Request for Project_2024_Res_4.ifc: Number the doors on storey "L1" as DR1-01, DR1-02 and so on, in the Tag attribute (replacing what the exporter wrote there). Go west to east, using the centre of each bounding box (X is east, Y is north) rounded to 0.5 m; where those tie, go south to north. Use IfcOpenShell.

First a look at what the model holds.

```python
import ifcopenshell
import ifcopenshell.util.element
import ifcopenshell.util.placement

model = ifcopenshell.open("Project_2024_Res_4.ifc")
print(model.schema)
storey = next(s for s in model.by_type("IfcBuildingStorey") if s.Name == "L1")
doors = [e for e in ifcopenshell.util.element.get_decomposition(storey) if e.is_a("IfcDoor")]
for e in sorted(doors, key=lambda e: e.id()):
    origin = ifcopenshell.util.placement.get_local_placement(e.ObjectPlacement)[:3, 3]
    print(e.id(), e.Tag, e.Name, origin.round(2) + 0.0, sep=" | ")
```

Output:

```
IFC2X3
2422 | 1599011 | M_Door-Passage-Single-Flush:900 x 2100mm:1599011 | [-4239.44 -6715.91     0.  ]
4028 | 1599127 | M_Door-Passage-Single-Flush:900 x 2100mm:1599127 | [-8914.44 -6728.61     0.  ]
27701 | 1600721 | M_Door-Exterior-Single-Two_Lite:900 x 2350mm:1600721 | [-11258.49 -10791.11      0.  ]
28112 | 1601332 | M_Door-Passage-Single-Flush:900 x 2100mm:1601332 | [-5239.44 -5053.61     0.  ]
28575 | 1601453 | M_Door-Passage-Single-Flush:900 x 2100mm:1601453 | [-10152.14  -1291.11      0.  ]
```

```python
import ifcopenshell
import ifcopenshell.geom
import ifcopenshell.util.element
import ifcopenshell.util.shape

model = ifcopenshell.open("Project_2024_Res_4.ifc")
settings = ifcopenshell.geom.settings()
settings.set("use-world-coords", True)


def centre(element):
    shape = ifcopenshell.geom.create_shape(settings, element)
    return ifcopenshell.util.shape.get_bbox_centroid(shape.geometry)


storey = next(s for s in model.by_type("IfcBuildingStorey") if s.Name == "L1")
doors = [e for e in ifcopenshell.util.element.get_decomposition(storey) if e.is_a("IfcDoor")]

# Insertion points can sit at a corner or the storey origin, so sort by the geometry (in metres).
centres = {e: centre(e) for e in doors}
doors.sort(key=lambda e: (round(centres[e][0] / 0.5), centres[e][1]))

for i, e in enumerate(doors, start=1):
    number = f"DR1-{i:02d}"
    e.Tag = number
    print(e.id(), number)

model.write("Project_2024_Res_4_v2.ifc")
```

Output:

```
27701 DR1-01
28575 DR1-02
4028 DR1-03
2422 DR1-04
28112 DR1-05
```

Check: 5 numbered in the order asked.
